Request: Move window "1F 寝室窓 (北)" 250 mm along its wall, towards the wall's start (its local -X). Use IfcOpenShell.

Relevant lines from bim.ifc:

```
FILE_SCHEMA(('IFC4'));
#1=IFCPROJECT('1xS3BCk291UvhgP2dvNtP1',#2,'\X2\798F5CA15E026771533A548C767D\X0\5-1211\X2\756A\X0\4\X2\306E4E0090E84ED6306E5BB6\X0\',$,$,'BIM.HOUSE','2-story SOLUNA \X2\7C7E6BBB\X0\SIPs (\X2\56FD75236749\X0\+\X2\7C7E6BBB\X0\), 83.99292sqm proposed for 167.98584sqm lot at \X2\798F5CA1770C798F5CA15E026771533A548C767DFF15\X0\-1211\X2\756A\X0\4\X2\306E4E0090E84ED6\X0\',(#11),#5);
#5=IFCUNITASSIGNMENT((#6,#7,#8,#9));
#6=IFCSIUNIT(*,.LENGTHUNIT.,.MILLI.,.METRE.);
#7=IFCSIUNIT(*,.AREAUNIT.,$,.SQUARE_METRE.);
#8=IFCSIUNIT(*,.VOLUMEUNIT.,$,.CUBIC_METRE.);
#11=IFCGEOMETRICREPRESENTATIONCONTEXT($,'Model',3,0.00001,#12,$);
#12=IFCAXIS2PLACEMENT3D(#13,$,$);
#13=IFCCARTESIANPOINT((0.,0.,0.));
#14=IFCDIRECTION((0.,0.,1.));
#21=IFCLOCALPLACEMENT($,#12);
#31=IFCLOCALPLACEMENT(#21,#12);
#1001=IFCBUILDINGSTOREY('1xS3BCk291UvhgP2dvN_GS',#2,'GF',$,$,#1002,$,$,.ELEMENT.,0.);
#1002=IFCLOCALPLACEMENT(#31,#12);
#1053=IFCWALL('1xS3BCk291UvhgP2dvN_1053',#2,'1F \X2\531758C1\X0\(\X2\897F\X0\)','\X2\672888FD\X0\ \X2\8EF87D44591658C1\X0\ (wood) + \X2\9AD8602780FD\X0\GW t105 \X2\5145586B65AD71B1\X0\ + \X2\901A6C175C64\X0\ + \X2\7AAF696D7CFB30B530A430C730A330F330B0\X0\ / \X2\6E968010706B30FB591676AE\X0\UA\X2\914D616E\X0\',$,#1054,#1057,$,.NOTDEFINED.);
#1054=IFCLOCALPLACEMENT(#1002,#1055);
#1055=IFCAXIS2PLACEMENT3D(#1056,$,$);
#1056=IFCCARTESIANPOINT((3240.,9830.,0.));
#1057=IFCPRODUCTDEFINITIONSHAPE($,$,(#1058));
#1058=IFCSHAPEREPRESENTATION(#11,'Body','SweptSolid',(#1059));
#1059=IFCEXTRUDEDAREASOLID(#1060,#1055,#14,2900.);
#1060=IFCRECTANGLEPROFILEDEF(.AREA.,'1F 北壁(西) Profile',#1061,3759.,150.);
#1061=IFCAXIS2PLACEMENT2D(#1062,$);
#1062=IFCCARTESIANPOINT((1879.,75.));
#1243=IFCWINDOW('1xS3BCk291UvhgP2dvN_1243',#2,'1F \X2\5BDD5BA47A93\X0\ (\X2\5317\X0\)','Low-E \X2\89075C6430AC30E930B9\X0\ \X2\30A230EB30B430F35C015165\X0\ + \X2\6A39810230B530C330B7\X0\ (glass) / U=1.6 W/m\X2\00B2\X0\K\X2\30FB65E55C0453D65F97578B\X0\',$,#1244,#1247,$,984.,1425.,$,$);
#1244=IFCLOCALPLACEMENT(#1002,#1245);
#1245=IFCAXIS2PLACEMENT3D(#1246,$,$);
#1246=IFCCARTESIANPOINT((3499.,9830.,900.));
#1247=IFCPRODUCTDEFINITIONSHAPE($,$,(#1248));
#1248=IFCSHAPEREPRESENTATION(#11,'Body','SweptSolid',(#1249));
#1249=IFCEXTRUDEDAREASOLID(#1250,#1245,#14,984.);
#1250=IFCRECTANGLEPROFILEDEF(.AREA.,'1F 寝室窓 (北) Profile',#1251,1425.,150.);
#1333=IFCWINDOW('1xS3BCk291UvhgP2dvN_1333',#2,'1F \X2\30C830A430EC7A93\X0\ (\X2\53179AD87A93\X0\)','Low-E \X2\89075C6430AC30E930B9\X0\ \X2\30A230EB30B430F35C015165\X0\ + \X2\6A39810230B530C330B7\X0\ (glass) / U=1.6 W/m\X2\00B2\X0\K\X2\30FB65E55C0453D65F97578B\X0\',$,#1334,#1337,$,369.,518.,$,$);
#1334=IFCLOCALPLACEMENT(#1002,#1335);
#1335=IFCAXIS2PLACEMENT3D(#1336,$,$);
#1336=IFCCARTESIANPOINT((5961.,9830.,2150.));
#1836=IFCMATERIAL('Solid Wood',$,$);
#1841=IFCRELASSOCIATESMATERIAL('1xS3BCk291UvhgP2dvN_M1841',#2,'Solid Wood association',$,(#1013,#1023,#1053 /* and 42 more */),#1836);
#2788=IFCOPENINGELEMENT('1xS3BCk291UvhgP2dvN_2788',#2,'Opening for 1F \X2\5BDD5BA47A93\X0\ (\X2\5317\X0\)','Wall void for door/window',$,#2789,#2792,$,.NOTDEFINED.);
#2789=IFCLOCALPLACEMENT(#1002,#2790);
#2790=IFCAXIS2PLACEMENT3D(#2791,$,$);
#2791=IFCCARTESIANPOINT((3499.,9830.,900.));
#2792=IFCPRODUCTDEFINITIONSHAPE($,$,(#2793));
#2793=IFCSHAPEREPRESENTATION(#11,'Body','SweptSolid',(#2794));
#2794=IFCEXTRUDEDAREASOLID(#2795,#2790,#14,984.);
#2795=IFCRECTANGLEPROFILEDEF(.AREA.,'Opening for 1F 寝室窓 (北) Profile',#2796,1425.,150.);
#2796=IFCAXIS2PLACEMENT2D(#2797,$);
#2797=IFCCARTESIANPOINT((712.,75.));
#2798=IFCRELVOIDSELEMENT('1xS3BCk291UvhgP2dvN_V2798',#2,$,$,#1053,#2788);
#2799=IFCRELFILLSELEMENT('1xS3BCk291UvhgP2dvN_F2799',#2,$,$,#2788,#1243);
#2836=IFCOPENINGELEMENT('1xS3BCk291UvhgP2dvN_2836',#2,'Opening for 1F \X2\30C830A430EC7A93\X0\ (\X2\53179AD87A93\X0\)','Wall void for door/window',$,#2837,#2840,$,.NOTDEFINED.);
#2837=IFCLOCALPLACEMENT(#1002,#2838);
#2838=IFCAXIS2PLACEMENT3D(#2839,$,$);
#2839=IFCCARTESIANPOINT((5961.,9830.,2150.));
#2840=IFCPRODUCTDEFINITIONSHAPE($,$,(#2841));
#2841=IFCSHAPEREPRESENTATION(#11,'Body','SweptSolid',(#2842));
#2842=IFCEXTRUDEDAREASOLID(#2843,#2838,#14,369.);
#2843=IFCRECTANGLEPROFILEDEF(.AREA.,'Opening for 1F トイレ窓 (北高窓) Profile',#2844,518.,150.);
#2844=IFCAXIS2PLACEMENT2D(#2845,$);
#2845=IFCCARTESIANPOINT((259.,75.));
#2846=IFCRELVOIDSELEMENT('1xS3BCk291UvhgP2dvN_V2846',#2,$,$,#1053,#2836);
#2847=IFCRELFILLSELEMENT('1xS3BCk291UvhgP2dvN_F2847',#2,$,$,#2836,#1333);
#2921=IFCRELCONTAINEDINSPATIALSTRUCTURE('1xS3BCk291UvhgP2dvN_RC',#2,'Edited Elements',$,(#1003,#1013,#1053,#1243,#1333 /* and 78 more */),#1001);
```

```python
import ifcopenshell
import ifcopenshell.api.geometry
import ifcopenshell.util.placement

model = ifcopenshell.open("bim.ifc")

window = model.by_guid("1xS3BCk291UvhgP2dvN_1243")
opening = window.FillsVoids[0].RelatingOpeningElement
wall = opening.VoidsElements[0].RelatingBuildingElement

wall_matrix = ifcopenshell.util.placement.get_local_placement(wall.ObjectPlacement)
shift = wall_matrix[:3, 0] * -250.0
before = ifcopenshell.util.placement.get_local_placement(window.ObjectPlacement)[:3, 3].copy()

# The window is not placed relative to its opening, so move both.
for product in (opening, window):
    matrix = ifcopenshell.util.placement.get_local_placement(product.ObjectPlacement)
    matrix[:3, 3] += shift
    ifcopenshell.api.geometry.edit_object_placement(model, product=product, matrix=matrix, is_si=False)

after = ifcopenshell.util.placement.get_local_placement(window.ObjectPlacement)[:3, 3]
print("window moved by", (after - before).round(3) + 0.0)

model.write("bim_edited.ifc")
```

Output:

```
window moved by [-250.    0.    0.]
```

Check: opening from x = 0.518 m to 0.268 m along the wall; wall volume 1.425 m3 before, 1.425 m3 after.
